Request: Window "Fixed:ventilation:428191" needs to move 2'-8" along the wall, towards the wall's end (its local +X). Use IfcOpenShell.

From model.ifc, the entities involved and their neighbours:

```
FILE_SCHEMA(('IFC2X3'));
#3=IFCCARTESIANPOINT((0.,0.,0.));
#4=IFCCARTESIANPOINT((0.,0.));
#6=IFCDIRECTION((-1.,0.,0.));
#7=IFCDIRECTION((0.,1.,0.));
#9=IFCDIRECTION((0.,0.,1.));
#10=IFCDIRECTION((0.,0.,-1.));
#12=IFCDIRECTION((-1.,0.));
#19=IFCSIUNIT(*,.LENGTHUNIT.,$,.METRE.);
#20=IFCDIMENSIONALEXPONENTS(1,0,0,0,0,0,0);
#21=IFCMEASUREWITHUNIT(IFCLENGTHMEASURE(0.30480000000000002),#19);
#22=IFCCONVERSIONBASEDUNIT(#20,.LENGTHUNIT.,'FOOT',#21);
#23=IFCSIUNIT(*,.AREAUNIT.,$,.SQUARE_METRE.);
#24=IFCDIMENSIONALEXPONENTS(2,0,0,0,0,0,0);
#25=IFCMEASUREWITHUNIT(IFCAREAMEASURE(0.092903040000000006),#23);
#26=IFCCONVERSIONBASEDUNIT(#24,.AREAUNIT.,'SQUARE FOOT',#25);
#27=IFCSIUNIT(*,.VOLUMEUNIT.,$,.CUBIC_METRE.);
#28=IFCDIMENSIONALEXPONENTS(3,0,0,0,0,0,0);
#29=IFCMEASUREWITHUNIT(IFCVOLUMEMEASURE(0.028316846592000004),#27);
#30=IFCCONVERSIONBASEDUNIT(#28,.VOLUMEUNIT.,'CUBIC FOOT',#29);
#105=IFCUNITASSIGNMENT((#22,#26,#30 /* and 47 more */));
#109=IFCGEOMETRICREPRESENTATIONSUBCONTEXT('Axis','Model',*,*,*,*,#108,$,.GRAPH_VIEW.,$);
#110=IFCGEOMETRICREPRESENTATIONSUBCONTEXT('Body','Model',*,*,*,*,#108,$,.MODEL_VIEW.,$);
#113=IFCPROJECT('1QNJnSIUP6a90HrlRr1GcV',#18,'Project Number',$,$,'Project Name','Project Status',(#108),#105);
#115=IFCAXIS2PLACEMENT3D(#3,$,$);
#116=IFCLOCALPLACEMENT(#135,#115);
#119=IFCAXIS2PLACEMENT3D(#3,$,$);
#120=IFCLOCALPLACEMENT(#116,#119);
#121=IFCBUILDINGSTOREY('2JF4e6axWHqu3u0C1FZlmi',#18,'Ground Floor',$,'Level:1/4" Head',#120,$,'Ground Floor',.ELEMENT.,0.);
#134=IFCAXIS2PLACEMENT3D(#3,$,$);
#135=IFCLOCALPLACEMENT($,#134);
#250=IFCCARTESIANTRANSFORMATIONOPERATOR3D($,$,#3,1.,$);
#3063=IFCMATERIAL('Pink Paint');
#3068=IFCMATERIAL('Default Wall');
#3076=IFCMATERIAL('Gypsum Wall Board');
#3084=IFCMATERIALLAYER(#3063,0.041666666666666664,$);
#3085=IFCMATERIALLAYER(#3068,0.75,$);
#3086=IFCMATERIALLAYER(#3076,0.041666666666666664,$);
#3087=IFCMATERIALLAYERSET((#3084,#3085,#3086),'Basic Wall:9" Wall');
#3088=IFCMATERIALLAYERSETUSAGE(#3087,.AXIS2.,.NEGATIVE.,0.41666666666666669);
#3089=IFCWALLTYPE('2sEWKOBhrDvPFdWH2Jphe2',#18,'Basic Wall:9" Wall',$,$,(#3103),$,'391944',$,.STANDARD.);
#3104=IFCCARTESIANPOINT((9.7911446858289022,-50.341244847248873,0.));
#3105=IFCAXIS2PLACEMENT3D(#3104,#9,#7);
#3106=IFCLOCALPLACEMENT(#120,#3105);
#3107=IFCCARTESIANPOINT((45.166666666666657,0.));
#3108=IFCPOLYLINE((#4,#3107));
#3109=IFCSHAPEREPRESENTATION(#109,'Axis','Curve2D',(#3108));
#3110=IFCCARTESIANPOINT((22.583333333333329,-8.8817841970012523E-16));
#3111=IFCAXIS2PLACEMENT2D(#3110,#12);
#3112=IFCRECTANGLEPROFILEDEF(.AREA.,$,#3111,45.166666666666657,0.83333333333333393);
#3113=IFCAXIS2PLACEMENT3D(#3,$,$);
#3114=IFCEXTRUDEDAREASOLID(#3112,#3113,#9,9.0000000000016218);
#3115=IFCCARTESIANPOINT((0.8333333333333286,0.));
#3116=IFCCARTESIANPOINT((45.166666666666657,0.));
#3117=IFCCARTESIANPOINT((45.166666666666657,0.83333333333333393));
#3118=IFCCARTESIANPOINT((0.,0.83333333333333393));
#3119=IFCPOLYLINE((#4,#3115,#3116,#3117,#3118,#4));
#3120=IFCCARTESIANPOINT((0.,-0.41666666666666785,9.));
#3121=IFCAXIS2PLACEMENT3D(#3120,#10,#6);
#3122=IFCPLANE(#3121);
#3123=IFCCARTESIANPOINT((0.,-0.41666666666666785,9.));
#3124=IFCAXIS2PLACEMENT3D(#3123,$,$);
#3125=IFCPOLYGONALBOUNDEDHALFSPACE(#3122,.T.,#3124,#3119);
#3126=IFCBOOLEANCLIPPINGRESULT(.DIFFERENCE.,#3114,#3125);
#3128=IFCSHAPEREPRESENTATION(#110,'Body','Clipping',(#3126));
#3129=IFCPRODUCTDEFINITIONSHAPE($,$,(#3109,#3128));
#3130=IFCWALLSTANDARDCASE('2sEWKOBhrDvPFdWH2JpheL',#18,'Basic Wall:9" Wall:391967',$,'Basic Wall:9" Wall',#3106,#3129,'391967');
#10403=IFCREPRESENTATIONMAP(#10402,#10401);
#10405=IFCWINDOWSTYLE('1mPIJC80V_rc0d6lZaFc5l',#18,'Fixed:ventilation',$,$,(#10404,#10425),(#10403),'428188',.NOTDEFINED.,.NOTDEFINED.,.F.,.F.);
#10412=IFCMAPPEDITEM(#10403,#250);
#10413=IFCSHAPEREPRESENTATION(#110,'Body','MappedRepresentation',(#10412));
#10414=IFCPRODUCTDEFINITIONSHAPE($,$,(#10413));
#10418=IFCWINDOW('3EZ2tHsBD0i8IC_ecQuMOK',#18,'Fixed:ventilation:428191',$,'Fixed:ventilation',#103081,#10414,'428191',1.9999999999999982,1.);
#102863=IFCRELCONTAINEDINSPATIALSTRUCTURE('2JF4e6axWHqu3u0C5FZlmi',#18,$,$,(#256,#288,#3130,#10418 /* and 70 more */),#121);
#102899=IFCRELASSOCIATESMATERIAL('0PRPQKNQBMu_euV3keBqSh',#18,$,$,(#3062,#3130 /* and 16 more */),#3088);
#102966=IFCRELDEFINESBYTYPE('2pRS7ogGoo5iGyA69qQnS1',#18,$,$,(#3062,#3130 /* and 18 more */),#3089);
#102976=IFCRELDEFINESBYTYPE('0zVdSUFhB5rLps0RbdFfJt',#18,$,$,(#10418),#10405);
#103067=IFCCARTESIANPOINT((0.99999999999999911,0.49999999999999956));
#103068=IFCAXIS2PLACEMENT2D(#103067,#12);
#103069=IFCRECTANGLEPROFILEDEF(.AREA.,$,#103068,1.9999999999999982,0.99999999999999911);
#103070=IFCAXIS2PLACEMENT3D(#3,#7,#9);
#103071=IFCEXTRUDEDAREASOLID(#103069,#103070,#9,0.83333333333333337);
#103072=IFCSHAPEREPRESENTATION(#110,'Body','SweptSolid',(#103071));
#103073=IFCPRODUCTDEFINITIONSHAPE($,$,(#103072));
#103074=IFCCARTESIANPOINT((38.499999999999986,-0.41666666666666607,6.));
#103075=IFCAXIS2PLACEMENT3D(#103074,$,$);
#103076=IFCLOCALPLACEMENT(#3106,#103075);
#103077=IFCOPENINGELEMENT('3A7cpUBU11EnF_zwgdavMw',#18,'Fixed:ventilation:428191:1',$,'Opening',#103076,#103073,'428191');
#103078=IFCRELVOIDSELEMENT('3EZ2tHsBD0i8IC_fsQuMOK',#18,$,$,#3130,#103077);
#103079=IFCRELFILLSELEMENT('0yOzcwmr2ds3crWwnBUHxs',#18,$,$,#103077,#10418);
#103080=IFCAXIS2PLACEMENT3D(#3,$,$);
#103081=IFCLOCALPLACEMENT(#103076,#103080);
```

```python
import ifcopenshell
import ifcopenshell.api.geometry
import ifcopenshell.util.placement
import ifcopenshell.util.unit

model = ifcopenshell.open("model.ifc")
unit_scale = ifcopenshell.util.unit.calculate_unit_scale(model)

window = model.by_id(10418)
opening = window.FillsVoids[0].RelatingOpeningElement
wall = opening.VoidsElements[0].RelatingBuildingElement

wall_matrix = ifcopenshell.util.placement.get_local_placement(wall.ObjectPlacement)
shift = wall_matrix[:3, 0] * 32 * 0.0254 / unit_scale
before = ifcopenshell.util.placement.get_local_placement(window.ObjectPlacement)[:3, 3].copy()

# The window is placed relative to its opening, so it follows when the opening moves.
matrix = ifcopenshell.util.placement.get_local_placement(opening.ObjectPlacement)
matrix[:3, 3] += shift
ifcopenshell.api.geometry.edit_object_placement(
    model, product=opening, matrix=matrix, is_si=False, should_transform_children=True
)

after = ifcopenshell.util.placement.get_local_placement(window.ObjectPlacement)[:3, 3]
print("window moved by", (after - before).round(3) + 0.0)

model.write("model_updated.ifc")
```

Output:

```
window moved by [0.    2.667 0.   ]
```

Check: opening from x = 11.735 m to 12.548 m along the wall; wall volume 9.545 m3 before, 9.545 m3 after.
